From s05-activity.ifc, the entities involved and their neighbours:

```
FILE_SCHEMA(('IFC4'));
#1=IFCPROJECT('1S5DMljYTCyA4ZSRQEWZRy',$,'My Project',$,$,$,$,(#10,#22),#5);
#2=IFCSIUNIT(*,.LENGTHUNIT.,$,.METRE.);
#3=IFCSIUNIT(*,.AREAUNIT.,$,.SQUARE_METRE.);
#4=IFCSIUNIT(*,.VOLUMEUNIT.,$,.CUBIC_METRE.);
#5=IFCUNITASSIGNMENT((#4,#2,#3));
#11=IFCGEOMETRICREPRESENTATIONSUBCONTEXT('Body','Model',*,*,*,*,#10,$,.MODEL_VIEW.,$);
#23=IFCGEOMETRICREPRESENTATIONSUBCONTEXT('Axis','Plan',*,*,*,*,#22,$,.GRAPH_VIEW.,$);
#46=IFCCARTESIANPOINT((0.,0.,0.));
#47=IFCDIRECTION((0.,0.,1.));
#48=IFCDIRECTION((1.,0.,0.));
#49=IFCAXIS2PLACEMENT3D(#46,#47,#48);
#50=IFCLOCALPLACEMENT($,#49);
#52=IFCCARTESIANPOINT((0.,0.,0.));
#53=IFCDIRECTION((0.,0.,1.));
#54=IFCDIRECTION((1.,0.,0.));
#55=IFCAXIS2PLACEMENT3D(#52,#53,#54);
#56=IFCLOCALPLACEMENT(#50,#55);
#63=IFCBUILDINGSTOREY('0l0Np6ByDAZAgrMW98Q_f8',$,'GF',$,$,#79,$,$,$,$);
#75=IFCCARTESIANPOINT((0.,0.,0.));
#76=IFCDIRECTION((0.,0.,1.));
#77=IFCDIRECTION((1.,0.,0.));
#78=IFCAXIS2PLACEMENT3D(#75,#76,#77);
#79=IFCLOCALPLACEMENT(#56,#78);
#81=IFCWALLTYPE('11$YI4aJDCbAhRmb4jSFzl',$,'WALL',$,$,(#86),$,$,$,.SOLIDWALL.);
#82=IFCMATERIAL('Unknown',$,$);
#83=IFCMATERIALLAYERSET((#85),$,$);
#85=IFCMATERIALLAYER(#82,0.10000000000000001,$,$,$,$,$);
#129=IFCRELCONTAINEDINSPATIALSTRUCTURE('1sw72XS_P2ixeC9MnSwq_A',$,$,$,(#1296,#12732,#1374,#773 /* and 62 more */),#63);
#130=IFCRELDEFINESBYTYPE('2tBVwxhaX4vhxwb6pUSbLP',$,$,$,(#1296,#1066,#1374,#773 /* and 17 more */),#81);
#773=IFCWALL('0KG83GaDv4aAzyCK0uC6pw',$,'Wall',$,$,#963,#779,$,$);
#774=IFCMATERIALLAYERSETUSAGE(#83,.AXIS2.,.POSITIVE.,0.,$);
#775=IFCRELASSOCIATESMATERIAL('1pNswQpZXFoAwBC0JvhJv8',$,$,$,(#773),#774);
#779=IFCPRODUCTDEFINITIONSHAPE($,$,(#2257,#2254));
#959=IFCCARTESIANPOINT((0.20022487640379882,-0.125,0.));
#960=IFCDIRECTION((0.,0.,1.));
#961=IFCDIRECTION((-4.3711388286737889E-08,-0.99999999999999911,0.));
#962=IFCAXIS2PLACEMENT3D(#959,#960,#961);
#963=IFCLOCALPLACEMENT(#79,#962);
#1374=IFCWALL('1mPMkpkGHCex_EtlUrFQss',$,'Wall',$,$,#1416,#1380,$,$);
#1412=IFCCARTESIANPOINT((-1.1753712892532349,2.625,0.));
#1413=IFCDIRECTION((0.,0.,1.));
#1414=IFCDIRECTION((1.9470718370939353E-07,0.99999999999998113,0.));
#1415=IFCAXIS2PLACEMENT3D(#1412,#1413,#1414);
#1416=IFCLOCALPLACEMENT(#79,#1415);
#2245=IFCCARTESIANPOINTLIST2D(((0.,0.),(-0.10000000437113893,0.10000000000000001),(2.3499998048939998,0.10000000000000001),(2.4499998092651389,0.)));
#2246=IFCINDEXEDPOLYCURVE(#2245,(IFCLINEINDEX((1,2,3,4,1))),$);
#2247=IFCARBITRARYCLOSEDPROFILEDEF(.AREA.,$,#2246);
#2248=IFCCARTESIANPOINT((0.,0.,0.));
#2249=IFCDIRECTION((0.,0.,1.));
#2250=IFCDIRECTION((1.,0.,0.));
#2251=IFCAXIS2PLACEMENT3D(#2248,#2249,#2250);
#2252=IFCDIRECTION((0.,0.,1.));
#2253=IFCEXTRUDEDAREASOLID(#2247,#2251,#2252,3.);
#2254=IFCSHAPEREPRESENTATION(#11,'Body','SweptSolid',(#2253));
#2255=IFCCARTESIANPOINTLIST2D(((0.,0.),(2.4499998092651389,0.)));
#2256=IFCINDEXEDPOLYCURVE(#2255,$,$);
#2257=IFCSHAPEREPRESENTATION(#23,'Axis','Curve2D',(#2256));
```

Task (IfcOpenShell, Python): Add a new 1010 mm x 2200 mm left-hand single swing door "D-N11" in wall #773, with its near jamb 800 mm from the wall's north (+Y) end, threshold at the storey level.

```python
import numpy as np
import ifcopenshell
import ifcopenshell.api.feature
import ifcopenshell.api.geometry
import ifcopenshell.api.root
import ifcopenshell.api.spatial
import ifcopenshell.geom
import ifcopenshell.util.element
import ifcopenshell.util.placement
import ifcopenshell.util.representation
import ifcopenshell.util.shape
import ifcopenshell.util.unit

model = ifcopenshell.open("s05-activity.ifc")
unit_scale = ifcopenshell.util.unit.calculate_unit_scale(model)
settings = ifcopenshell.geom.settings()


def volume(element):
    """Net volume in cubic metres, openings subtracted."""
    shape = ifcopenshell.geom.create_shape(settings, element)
    return ifcopenshell.util.shape.get_volume(shape.geometry)


wall = model.by_guid("0KG83GaDv4aAzyCK0uC6pw")
storey = ifcopenshell.util.element.get_container(wall, ifc_class="IfcBuildingStorey")
context = ifcopenshell.util.representation.get_context(model, "Model", "Body", "MODEL_VIEW")
before = volume(wall)

width, height, from_end, sill = 1.01, 2.2, 0.8, 0.0  # metres

# The wall runs along its own X axis, and the end named is its -X end.
wall_shape = ifcopenshell.geom.create_shape(settings, wall)
x, y, z = ifcopenshell.util.shape.get_vertices(wall_shape.geometry).T
start = x.min() + from_end
face, thickness = float(y.min()), float(y.max() - y.min())
wall_matrix = ifcopenshell.util.placement.get_local_placement(wall.ObjectPlacement)
level = ifcopenshell.util.placement.get_local_placement(storey.ObjectPlacement)[2, 3]


def in_wall(x, y):
    """Placement at x, y metres in the wall's axes, at sill height."""
    matrix = wall_matrix.copy()
    matrix[:, 3] = wall_matrix @ np.array([x / unit_scale, y / unit_scale, 0.0, 1.0])
    matrix[2, 3] = level + sill / unit_scale
    return matrix


# Opening: a box that overshoots both wall faces by 50 mm.
opening = ifcopenshell.api.root.create_entity(model, ifc_class="IfcOpeningElement", predefined_type="OPENING")
box = ifcopenshell.api.geometry.add_wall_representation(
    model, context=context, length=width, height=height, thickness=thickness + 0.1
)
ifcopenshell.api.geometry.assign_representation(model, product=opening, representation=box)
ifcopenshell.api.geometry.edit_object_placement(model, product=opening, matrix=in_wall(start, face - 0.05), is_si=False)
ifcopenshell.api.feature.add_feature(model, feature=opening, element=wall)

door = ifcopenshell.api.root.create_entity(model, ifc_class="IfcDoor", name="D-N11", predefined_type="DOOR")
door.OverallWidth, door.OverallHeight = width / unit_scale, height / unit_scale
door.OperationType = "SINGLE_SWING_LEFT"
body = ifcopenshell.api.geometry.add_door_representation(
    model,
    context=context,
    overall_width=door.OverallWidth,
    overall_height=door.OverallHeight,
    operation_type="SINGLE_SWING_LEFT",
    lining_properties={"LiningDepth": thickness / unit_scale, "ThresholdDepth": thickness / unit_scale},
)
ifcopenshell.api.geometry.assign_representation(model, product=door, representation=body)
ifcopenshell.api.spatial.assign_container(model, products=[door], relating_structure=storey)
ifcopenshell.api.feature.add_filling(model, opening=opening, element=door)

# The lining spans the wall, so the door starts at the wall face.
ifcopenshell.api.geometry.edit_object_placement(model, product=door, matrix=in_wall(start, face), is_si=False)

after = volume(wall)

print(f"wall volume {before:.3f} -> {after:.3f} m3")

model.write("s05-activity_v2.ifc")
```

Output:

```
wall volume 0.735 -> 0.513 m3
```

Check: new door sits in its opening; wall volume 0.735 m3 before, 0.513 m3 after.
